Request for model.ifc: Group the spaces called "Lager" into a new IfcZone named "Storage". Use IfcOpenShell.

First a look at what the model holds.

```python
import ifcopenshell

model = ifcopenshell.open("model.ifc")
print(model.schema)
seen = {}
for space in model.by_type("IfcSpace"):
    seen[space.LongName] = seen.get(space.LongName, 0) + 1
for name, count in sorted(seen.items(), key=str):
    print(count, "x", name)
print("zones:", [z.Name for z in model.by_type("IfcZone")][:20])
```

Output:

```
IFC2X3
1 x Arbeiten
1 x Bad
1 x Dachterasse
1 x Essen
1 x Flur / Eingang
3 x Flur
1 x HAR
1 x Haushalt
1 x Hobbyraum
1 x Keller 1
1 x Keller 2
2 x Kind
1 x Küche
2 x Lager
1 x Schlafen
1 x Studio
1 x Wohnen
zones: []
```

```python
import ifcopenshell
import ifcopenshell.api.group
import ifcopenshell.api.root

model = ifcopenshell.open("model.ifc")

names = {"Lager"}
spaces = [s for s in model.by_type("IfcSpace") if s.LongName in names]

zone = ifcopenshell.api.root.create_entity(model, ifc_class="IfcZone", name="Storage")
ifcopenshell.api.group.assign_group(model, products=spaces, group=zone)
print(len(spaces), "spaces in", zone.Name)

model.write("model_updated.ifc")
```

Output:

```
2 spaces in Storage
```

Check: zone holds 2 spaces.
